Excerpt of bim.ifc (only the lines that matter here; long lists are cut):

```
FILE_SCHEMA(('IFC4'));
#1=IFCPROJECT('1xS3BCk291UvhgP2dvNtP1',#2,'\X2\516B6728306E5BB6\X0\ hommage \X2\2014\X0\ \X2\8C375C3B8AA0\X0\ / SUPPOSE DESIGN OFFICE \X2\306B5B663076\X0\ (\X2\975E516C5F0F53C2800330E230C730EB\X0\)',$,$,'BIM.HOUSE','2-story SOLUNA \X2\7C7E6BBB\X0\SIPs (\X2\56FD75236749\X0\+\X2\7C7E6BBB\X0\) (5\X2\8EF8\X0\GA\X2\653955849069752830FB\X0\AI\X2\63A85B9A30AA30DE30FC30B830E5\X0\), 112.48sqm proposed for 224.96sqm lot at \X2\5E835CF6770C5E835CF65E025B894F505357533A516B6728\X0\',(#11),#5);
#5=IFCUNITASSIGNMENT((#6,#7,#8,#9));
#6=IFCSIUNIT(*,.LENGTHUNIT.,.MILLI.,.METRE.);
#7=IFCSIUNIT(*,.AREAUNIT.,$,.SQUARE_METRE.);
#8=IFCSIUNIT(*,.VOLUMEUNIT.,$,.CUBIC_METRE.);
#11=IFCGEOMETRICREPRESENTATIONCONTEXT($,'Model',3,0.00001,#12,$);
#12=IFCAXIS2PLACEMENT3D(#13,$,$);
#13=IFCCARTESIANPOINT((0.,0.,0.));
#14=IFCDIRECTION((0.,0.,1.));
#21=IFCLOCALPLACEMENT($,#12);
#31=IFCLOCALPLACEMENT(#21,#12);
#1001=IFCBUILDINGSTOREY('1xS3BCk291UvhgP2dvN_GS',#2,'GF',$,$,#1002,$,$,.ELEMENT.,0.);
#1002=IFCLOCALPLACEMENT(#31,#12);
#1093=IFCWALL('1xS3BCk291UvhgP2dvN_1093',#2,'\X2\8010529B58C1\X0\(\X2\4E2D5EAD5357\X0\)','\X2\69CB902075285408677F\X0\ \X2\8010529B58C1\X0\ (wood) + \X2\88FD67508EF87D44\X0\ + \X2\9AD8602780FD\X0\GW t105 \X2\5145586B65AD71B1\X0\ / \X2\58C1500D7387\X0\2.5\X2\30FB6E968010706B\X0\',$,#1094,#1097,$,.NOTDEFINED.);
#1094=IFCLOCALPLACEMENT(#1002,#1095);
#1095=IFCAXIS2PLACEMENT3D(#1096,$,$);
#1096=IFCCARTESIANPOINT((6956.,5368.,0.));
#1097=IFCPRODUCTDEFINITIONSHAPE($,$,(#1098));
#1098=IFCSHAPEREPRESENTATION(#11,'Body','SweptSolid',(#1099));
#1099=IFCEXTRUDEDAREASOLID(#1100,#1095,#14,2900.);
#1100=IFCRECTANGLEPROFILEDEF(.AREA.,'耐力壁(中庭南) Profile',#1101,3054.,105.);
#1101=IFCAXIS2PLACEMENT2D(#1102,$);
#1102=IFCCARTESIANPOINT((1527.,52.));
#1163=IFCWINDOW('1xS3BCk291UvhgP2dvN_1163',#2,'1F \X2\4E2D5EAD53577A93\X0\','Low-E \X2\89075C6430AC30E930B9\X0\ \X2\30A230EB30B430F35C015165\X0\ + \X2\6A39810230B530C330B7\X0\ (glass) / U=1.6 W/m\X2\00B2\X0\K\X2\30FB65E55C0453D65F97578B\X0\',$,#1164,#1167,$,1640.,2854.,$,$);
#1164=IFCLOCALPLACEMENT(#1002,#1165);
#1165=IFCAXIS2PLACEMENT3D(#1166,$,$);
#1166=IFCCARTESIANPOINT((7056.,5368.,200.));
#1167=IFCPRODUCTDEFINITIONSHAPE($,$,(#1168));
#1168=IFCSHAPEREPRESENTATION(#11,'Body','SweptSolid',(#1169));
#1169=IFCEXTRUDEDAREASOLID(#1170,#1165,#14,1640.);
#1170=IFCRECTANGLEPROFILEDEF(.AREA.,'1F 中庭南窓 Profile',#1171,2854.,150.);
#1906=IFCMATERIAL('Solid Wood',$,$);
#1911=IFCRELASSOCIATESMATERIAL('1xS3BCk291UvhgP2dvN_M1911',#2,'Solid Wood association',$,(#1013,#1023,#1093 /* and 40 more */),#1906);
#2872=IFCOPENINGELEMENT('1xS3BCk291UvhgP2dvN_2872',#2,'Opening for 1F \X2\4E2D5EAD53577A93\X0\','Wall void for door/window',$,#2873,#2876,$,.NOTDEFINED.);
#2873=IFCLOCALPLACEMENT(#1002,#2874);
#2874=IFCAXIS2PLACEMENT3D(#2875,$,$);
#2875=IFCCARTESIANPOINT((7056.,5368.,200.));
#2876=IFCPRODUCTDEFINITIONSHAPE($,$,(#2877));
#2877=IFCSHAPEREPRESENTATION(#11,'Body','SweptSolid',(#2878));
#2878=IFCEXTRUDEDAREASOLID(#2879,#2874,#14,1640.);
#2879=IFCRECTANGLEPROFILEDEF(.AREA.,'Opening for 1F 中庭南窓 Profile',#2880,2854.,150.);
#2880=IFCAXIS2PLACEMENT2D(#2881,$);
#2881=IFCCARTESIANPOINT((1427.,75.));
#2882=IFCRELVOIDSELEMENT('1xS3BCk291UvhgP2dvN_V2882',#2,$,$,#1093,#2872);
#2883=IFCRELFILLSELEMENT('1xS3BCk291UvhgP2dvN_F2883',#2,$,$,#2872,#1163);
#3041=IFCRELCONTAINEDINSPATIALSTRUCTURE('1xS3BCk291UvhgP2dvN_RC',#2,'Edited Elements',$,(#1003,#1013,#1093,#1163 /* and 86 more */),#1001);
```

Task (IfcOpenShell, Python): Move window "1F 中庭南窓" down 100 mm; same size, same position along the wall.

```python
import numpy as np
import ifcopenshell
import ifcopenshell.api.geometry
import ifcopenshell.util.placement
import ifcopenshell.util.unit

model = ifcopenshell.open("bim.ifc")
unit_scale = ifcopenshell.util.unit.calculate_unit_scale(model)

window = model.by_id(1163)
opening = window.FillsVoids[0].RelatingOpeningElement
dz = -0.1 / unit_scale

shift = np.array([0.0, 0.0, dz])
# The window is not placed relative to its opening, so move both.
for product in (opening, window):
    matrix = ifcopenshell.util.placement.get_local_placement(product.ObjectPlacement)
    matrix[:3, 3] += shift
    ifcopenshell.api.geometry.edit_object_placement(model, product=product, matrix=matrix, is_si=False)

print(f"moved by {dz * unit_scale:+.3f} m")

model.write("bim_edited.ifc")
```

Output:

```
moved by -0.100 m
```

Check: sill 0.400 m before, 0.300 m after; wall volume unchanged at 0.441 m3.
